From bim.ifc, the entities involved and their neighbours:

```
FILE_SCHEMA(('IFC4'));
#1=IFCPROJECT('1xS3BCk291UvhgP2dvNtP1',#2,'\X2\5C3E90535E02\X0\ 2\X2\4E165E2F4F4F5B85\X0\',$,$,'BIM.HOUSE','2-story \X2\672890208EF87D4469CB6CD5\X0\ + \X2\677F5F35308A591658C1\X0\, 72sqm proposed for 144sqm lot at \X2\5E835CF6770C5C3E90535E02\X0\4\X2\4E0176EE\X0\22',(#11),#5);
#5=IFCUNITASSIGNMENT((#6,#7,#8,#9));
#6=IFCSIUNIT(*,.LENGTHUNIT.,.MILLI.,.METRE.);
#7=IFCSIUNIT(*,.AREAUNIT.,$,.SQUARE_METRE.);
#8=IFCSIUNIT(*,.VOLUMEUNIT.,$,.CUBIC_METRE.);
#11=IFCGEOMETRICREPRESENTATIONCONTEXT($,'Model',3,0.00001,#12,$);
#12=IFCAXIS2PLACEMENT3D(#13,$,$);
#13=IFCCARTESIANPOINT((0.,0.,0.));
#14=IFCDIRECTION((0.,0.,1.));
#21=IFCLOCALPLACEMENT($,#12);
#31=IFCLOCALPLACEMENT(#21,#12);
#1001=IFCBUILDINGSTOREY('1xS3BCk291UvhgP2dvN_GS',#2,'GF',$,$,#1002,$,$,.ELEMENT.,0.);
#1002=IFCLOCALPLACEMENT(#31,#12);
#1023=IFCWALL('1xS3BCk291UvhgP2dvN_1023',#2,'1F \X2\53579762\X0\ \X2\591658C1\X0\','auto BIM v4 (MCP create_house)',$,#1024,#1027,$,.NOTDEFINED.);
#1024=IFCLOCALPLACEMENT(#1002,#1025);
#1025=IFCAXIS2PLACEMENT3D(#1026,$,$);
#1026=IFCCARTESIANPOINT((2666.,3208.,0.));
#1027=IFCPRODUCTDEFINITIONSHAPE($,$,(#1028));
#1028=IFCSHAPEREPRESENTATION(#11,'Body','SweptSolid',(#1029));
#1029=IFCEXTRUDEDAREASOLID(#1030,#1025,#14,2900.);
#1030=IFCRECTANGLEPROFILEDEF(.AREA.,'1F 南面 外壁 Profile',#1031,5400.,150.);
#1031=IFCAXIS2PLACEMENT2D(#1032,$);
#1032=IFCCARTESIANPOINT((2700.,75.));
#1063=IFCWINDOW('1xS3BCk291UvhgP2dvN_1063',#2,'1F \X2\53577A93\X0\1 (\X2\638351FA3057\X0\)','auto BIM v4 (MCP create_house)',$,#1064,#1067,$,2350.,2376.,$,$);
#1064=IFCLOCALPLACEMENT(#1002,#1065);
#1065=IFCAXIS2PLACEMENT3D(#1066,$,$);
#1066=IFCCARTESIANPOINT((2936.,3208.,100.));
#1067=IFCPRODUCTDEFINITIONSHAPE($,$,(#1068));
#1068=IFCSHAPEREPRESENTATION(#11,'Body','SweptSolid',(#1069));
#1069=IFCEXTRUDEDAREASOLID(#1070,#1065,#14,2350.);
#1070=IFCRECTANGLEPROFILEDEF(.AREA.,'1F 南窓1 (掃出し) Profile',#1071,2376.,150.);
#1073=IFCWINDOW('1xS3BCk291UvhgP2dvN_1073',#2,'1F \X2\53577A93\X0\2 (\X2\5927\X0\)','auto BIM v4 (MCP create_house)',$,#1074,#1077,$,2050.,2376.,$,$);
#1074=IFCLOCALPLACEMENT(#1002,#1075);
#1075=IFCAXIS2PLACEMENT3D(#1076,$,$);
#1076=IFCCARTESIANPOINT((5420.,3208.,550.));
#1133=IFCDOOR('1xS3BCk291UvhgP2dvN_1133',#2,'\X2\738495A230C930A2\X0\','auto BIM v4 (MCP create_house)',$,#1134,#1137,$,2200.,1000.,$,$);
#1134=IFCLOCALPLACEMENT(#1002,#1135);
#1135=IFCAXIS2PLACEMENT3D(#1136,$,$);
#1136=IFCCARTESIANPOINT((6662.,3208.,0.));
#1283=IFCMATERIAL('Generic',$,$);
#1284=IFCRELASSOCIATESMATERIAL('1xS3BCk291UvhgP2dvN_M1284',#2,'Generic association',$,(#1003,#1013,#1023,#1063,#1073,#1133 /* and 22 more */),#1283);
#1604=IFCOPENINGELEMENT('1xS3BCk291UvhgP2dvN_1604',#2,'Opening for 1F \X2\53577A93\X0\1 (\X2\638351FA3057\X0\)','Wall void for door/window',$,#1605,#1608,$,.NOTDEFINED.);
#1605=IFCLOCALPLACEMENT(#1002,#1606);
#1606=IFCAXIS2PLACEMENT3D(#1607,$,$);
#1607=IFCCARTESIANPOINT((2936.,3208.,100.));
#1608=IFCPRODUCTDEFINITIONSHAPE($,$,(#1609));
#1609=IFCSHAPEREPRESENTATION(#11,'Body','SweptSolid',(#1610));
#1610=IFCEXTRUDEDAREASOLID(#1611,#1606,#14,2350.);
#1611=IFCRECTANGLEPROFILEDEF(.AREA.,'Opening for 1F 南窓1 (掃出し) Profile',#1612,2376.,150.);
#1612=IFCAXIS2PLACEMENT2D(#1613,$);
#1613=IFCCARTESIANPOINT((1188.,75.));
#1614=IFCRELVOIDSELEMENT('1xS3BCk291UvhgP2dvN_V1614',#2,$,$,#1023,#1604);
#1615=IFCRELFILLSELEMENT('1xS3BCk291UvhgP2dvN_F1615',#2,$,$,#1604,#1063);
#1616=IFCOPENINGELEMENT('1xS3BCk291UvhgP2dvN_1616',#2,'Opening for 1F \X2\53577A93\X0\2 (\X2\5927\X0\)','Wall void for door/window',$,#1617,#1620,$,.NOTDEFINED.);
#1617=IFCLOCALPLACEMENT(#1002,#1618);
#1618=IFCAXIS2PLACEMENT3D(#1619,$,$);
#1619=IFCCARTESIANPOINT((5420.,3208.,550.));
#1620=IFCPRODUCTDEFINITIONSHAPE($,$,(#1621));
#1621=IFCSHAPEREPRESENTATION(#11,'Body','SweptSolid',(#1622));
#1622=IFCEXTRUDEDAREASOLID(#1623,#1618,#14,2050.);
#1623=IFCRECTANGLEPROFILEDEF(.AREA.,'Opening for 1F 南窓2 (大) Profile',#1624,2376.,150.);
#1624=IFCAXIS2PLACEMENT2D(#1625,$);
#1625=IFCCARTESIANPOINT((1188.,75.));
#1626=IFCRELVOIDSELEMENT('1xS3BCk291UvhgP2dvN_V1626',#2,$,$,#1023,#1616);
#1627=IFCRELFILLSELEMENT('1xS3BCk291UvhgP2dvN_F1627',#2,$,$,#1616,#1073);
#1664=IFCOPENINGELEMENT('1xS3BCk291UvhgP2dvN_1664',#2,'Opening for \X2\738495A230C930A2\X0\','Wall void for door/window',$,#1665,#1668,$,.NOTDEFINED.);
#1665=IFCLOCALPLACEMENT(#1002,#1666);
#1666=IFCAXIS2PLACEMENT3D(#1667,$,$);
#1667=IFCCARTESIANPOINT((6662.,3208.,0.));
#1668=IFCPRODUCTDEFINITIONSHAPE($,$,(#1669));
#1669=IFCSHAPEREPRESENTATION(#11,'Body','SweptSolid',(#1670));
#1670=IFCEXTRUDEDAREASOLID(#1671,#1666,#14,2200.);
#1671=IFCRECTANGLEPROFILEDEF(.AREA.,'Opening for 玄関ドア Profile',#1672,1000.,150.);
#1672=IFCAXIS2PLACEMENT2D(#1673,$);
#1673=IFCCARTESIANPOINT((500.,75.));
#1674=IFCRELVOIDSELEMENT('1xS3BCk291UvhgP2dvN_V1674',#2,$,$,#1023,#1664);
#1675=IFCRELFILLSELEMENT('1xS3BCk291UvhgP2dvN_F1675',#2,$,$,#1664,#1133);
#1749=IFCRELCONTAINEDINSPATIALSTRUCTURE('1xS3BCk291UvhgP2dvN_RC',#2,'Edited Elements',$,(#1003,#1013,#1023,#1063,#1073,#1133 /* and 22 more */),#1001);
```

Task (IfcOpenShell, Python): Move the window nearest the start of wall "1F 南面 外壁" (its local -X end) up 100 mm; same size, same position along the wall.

```python
import numpy as np
import ifcopenshell
import ifcopenshell.api.geometry
import ifcopenshell.util.placement
import ifcopenshell.util.unit

model = ifcopenshell.open("bim.ifc")
unit_scale = ifcopenshell.util.unit.calculate_unit_scale(model)

window = model.by_id(1063)
opening = window.FillsVoids[0].RelatingOpeningElement
dz = 100.0

shift = np.array([0.0, 0.0, dz])
# The window is not placed relative to its opening, so move both.
for product in (opening, window):
    matrix = ifcopenshell.util.placement.get_local_placement(product.ObjectPlacement)
    matrix[:3, 3] += shift
    ifcopenshell.api.geometry.edit_object_placement(model, product=product, matrix=matrix, is_si=False)

print(f"moved by {dz * unit_scale:+.3f} m")

model.write("bim_edited.ifc")
```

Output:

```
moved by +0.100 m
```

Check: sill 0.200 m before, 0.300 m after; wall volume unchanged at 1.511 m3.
